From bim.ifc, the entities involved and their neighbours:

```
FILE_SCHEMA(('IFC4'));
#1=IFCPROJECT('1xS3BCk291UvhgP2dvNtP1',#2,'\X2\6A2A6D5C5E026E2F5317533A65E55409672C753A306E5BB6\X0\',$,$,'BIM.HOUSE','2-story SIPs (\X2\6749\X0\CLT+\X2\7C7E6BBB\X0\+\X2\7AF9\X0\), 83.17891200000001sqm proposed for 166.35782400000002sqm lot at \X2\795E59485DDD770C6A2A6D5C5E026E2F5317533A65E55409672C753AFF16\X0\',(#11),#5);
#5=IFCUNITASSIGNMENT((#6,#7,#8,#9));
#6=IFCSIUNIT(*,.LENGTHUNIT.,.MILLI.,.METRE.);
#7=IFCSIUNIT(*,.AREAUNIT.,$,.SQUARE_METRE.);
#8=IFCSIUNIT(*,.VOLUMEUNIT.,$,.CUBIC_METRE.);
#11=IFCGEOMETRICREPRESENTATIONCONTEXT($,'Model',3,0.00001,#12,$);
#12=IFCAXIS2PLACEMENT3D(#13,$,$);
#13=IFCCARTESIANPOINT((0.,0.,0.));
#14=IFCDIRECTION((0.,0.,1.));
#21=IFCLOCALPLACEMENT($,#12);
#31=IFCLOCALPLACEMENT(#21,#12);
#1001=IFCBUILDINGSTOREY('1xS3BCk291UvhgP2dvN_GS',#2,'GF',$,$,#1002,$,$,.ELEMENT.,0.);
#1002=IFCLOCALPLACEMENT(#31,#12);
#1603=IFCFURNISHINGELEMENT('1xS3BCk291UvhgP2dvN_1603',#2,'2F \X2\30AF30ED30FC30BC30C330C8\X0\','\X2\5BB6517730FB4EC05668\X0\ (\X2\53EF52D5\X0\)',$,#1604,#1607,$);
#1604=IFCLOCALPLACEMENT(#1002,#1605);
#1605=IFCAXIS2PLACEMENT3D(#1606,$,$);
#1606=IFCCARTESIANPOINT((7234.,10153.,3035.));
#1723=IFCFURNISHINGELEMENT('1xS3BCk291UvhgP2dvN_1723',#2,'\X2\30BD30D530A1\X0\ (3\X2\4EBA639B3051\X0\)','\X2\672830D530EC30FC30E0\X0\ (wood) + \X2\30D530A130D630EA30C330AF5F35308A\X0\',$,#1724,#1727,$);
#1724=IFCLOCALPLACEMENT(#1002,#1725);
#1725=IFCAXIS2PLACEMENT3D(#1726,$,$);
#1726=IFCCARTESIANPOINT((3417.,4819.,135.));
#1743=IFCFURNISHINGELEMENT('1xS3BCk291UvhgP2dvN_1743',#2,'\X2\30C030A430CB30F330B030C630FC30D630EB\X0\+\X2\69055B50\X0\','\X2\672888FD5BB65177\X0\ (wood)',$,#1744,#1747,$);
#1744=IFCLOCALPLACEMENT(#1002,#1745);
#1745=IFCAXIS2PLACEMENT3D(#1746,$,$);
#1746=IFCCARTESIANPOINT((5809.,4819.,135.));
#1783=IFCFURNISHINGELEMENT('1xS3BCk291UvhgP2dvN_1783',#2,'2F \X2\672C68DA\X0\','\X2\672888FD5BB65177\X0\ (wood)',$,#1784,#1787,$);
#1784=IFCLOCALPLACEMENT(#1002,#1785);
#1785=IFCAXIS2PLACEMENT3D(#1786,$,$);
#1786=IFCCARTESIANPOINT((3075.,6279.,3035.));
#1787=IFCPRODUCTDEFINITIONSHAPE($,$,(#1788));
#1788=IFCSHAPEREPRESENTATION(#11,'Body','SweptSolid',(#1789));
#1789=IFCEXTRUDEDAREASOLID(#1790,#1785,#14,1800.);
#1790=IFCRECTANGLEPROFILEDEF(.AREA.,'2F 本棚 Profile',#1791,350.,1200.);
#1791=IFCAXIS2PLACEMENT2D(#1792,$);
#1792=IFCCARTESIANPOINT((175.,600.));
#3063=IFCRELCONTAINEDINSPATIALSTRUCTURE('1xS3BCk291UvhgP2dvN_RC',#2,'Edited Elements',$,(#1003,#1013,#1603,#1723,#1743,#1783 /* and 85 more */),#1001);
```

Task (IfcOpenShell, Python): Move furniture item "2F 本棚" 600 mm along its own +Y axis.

```python
import ifcopenshell
import ifcopenshell.api.geometry
import ifcopenshell.util.placement
import ifcopenshell.util.unit

model = ifcopenshell.open("bim.ifc")
unit_scale = ifcopenshell.util.unit.calculate_unit_scale(model)

item = model.by_guid("1xS3BCk291UvhgP2dvN_1783")
matrix = ifcopenshell.util.placement.get_local_placement(item.ObjectPlacement)
matrix[:3, 3] += matrix[:3, 1] * 0.6 / unit_scale
ifcopenshell.api.geometry.edit_object_placement(model, product=item, matrix=matrix, is_si=False)

print(ifcopenshell.util.placement.get_local_placement(item.ObjectPlacement).round(3) + 0.0)

model.write("bim-out.ifc")
```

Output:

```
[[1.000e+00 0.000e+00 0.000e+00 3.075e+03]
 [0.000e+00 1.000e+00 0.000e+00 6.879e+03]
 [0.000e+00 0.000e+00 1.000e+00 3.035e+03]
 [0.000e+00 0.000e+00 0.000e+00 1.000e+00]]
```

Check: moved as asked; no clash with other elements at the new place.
